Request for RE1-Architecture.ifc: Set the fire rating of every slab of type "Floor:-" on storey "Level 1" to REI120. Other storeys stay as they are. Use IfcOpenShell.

First a look at what the model holds.

```python
import ifcopenshell
import ifcopenshell.util.element

model = ifcopenshell.open("RE1-Architecture.ifc")
print(model.schema)
storey = next(s for s in model.by_type("IfcBuildingStorey") if s.Name == "Level 1")
slabs = [e for e in ifcopenshell.util.element.get_decomposition(storey) if e.is_a("IfcSlab")]
seen = {}
for e in slabs:
    element_type = ifcopenshell.util.element.get_type(e)
    key = (element_type.Name if element_type != e and element_type else None, ifcopenshell.util.element.get_pset(e, "Pset_SlabCommon", "FireRating"))
    seen[key] = seen.get(key, 0) + 1
for (name, value), count in sorted(seen.items(), key=str):
    print(count, "x", name, "|", value)
```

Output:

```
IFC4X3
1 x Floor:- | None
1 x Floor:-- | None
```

```python
import ifcopenshell
import ifcopenshell.api.pset
import ifcopenshell.util.element

model = ifcopenshell.open("RE1-Architecture.ifc")

storey = next(s for s in model.by_type("IfcBuildingStorey") if s.Name == "Level 1")
slabs = [e for e in ifcopenshell.util.element.get_decomposition(storey) if e.is_a("IfcSlab")]

count = 0
for e in slabs:
    element_type = ifcopenshell.util.element.get_type(e)
    if element_type in (None, e) or element_type.Name != "Floor:-":
        continue
    # add_pset returns the element's existing set when there is one.
    pset = ifcopenshell.api.pset.add_pset(model, product=e, name="Pset_SlabCommon")
    ifcopenshell.api.pset.edit_pset(model, pset=pset, properties={"FireRating": "REI120"})
    count += 1

print(count, "slabs updated")

model.write("RE1-Architecture_edited.ifc")
```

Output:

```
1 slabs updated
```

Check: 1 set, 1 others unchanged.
